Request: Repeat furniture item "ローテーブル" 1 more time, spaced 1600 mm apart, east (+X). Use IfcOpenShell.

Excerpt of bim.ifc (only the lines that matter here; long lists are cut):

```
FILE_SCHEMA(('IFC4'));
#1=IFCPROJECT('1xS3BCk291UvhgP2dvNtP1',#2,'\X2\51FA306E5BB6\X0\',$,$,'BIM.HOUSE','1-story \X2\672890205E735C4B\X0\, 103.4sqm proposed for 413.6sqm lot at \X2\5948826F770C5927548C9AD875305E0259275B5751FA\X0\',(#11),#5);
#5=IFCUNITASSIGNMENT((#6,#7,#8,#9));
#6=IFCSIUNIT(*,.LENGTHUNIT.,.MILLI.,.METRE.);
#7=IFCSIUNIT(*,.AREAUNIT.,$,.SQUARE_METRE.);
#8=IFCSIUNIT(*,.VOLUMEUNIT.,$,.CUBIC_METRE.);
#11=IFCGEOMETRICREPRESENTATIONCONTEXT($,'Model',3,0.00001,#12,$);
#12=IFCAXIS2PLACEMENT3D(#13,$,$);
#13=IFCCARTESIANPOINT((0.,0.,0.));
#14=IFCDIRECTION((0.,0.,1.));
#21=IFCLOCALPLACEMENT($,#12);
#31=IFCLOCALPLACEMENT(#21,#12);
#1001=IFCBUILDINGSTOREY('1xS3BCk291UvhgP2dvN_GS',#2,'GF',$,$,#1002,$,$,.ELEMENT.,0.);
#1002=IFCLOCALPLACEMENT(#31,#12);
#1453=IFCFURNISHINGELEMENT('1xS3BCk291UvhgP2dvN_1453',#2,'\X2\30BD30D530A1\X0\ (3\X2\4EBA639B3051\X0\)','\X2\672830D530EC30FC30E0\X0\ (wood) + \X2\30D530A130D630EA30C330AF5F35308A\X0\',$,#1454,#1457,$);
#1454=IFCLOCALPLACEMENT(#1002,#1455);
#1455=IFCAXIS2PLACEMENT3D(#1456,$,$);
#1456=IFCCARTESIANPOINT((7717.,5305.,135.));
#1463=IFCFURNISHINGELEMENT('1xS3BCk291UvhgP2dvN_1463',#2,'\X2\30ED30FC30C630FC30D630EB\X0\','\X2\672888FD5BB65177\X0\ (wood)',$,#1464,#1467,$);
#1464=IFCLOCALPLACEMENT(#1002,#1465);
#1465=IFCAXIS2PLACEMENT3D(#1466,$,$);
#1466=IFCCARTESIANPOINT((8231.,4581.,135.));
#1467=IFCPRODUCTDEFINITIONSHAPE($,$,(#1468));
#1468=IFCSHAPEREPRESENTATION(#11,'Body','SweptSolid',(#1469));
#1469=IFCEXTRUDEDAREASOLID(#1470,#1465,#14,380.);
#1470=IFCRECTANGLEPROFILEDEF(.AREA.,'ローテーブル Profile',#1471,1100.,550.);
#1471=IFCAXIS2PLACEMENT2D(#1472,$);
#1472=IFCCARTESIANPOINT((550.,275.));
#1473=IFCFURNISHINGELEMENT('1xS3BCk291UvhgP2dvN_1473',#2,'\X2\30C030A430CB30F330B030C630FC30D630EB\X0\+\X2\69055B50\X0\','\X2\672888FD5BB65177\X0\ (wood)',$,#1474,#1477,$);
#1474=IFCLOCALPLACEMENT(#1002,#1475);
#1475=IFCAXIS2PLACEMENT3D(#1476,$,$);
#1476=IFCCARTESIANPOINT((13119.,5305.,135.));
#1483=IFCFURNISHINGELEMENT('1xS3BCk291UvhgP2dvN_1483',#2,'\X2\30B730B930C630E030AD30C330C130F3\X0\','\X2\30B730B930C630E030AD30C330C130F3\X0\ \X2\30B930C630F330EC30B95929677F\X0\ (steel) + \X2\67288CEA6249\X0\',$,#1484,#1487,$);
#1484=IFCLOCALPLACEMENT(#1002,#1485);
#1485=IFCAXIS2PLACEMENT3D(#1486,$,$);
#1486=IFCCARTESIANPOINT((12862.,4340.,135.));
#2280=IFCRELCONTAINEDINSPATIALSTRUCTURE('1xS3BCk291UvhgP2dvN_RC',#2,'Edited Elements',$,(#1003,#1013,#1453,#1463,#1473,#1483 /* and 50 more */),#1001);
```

```python
import numpy as np
import ifcopenshell
import ifcopenshell.api.geometry
import ifcopenshell.api.root
import ifcopenshell.util.element
import ifcopenshell.util.placement
import ifcopenshell.util.unit

model = ifcopenshell.open("bim.ifc")
unit_scale = ifcopenshell.util.unit.calculate_unit_scale(model)


def reuse_history(source, copy):
    """copy_class also copies each property set's owner history, people and application; keep the originals."""
    for rel in copy.IsDefinedBy:
        if rel.is_a("IfcRelDefinesByProperties") and (history := rel.RelatingPropertyDefinition.OwnerHistory):
            rel.RelatingPropertyDefinition.OwnerHistory = source.OwnerHistory
            ifcopenshell.util.element.remove_deep2(model, history)


source = model.by_id(1463)
base = ifcopenshell.util.placement.get_local_placement(source.ObjectPlacement)
step = np.array([1.0, 0.0, 0.0]) * 1.6 / unit_scale

for i in range(1, 2):
    copy = ifcopenshell.api.root.copy_class(model, product=source)
    copy.Representation = ifcopenshell.util.element.copy_deep(
        model, source.Representation, exclude=["IfcGeometricRepresentationContext", "IfcRepresentationMap"]
    )
    reuse_history(source, copy)
    matrix = base.copy()
    matrix[:3, 3] += i * step
    print("added at", matrix[:3, 3].round(3) + 0.0)
    ifcopenshell.api.geometry.edit_object_placement(model, product=copy, matrix=matrix, is_si=False)

model.write("bim_edited.ifc")
```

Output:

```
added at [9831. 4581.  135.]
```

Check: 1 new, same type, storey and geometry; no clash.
